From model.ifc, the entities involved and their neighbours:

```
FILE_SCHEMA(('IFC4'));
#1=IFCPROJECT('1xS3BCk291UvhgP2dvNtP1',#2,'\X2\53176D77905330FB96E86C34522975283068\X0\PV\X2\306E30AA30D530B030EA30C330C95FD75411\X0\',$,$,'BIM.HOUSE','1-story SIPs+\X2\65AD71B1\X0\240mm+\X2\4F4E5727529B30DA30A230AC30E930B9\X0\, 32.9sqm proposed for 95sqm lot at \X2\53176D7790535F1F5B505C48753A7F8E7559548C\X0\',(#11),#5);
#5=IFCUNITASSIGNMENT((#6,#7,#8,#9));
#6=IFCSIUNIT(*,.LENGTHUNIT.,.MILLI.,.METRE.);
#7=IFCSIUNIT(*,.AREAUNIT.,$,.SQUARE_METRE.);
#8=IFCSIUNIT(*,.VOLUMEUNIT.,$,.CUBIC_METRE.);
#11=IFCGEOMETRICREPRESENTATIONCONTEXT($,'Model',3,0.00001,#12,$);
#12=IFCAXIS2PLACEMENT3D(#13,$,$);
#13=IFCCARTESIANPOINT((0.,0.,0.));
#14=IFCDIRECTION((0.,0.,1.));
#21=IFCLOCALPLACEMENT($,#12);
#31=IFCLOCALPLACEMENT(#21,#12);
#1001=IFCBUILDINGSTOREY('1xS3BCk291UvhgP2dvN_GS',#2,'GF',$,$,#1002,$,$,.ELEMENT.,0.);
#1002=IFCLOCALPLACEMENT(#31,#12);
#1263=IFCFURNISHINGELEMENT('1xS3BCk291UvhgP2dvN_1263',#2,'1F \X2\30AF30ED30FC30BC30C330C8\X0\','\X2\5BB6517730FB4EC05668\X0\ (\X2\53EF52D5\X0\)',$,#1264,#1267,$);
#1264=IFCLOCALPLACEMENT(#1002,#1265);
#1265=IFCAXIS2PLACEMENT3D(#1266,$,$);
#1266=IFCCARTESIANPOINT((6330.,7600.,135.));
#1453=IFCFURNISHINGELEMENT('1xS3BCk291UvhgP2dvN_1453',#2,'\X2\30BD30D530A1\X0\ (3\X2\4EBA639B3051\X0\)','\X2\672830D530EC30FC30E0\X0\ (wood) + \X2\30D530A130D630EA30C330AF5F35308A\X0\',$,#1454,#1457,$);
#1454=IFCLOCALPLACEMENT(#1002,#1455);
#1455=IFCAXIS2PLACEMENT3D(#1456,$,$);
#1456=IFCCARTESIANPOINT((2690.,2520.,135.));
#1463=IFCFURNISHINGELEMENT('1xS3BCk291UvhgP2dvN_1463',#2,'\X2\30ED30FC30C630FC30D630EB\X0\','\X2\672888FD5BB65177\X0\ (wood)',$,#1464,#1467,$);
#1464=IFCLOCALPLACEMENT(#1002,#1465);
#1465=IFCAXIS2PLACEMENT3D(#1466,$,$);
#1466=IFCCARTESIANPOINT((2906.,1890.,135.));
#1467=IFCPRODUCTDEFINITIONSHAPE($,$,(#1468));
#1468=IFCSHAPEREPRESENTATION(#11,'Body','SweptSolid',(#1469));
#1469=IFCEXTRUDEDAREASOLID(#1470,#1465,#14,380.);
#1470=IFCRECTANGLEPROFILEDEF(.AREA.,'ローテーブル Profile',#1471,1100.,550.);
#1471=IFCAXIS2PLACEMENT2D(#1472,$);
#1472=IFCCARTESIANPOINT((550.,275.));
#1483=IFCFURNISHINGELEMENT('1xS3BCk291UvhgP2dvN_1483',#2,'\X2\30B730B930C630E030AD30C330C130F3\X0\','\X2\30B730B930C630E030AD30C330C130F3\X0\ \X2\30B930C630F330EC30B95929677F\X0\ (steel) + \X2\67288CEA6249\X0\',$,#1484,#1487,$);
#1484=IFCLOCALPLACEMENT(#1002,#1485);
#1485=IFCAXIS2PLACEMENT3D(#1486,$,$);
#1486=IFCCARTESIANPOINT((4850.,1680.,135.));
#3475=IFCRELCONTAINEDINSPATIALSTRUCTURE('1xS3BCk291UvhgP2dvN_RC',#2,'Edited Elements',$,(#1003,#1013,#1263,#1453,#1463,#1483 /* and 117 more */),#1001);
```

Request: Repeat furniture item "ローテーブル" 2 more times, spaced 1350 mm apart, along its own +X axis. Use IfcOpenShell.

```python
import ifcopenshell
import ifcopenshell.api.geometry
import ifcopenshell.api.root
import ifcopenshell.util.element
import ifcopenshell.util.placement
import ifcopenshell.util.unit

model = ifcopenshell.open("model.ifc")
unit_scale = ifcopenshell.util.unit.calculate_unit_scale(model)


def reuse_history(source, copy):
    """copy_class also copies each property set's owner history, people and application; keep the originals."""
    for rel in copy.IsDefinedBy:
        if rel.is_a("IfcRelDefinesByProperties") and (history := rel.RelatingPropertyDefinition.OwnerHistory):
            rel.RelatingPropertyDefinition.OwnerHistory = source.OwnerHistory
            ifcopenshell.util.element.remove_deep2(model, history)


source = model.by_guid("1xS3BCk291UvhgP2dvN_1463")
base = ifcopenshell.util.placement.get_local_placement(source.ObjectPlacement)
step = base[:3, 0] * 1.35 / unit_scale

for i in range(1, 3):
    copy = ifcopenshell.api.root.copy_class(model, product=source)
    copy.Representation = ifcopenshell.util.element.copy_deep(
        model, source.Representation, exclude=["IfcGeometricRepresentationContext", "IfcRepresentationMap"]
    )
    reuse_history(source, copy)
    matrix = base.copy()
    matrix[:3, 3] += i * step
    print("added at", matrix[:3, 3].round(3) + 0.0)
    ifcopenshell.api.geometry.edit_object_placement(model, product=copy, matrix=matrix, is_si=False)

model.write("model_updated.ifc")
```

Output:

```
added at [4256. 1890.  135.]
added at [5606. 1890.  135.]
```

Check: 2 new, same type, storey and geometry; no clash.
